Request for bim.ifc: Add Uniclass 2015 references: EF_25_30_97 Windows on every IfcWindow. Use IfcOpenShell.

First a look at what the model holds.

```python
import ifcopenshell

model = ifcopenshell.open("bim.ifc")
print(model.schema)
print("classifications:", [c.Name for c in model.by_type("IfcClassification")])
for ifc_class in ("IfcDoor", "IfcRoof", "IfcStair", "IfcWall", "IfcWindow"):
    print(ifc_class, len(model.by_type(ifc_class)))
```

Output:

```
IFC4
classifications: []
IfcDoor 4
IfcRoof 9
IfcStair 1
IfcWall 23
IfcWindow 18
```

```python
import ifcopenshell
import ifcopenshell.api.classification

model = ifcopenshell.open("bim.ifc")

system = ifcopenshell.api.classification.add_classification(model, classification="Uniclass 2015")

codes = {
    "IfcWindow": ("EF_25_30_97", "Windows"),
}
for ifc_class, (code, name) in codes.items():
    products = model.by_type(ifc_class)
    ifcopenshell.api.classification.add_reference(
        model, products=products, classification=system, identification=code, name=name
    )
    print(code, len(products))

model.write("bim_v2.ifc")
```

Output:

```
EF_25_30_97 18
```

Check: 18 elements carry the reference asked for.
